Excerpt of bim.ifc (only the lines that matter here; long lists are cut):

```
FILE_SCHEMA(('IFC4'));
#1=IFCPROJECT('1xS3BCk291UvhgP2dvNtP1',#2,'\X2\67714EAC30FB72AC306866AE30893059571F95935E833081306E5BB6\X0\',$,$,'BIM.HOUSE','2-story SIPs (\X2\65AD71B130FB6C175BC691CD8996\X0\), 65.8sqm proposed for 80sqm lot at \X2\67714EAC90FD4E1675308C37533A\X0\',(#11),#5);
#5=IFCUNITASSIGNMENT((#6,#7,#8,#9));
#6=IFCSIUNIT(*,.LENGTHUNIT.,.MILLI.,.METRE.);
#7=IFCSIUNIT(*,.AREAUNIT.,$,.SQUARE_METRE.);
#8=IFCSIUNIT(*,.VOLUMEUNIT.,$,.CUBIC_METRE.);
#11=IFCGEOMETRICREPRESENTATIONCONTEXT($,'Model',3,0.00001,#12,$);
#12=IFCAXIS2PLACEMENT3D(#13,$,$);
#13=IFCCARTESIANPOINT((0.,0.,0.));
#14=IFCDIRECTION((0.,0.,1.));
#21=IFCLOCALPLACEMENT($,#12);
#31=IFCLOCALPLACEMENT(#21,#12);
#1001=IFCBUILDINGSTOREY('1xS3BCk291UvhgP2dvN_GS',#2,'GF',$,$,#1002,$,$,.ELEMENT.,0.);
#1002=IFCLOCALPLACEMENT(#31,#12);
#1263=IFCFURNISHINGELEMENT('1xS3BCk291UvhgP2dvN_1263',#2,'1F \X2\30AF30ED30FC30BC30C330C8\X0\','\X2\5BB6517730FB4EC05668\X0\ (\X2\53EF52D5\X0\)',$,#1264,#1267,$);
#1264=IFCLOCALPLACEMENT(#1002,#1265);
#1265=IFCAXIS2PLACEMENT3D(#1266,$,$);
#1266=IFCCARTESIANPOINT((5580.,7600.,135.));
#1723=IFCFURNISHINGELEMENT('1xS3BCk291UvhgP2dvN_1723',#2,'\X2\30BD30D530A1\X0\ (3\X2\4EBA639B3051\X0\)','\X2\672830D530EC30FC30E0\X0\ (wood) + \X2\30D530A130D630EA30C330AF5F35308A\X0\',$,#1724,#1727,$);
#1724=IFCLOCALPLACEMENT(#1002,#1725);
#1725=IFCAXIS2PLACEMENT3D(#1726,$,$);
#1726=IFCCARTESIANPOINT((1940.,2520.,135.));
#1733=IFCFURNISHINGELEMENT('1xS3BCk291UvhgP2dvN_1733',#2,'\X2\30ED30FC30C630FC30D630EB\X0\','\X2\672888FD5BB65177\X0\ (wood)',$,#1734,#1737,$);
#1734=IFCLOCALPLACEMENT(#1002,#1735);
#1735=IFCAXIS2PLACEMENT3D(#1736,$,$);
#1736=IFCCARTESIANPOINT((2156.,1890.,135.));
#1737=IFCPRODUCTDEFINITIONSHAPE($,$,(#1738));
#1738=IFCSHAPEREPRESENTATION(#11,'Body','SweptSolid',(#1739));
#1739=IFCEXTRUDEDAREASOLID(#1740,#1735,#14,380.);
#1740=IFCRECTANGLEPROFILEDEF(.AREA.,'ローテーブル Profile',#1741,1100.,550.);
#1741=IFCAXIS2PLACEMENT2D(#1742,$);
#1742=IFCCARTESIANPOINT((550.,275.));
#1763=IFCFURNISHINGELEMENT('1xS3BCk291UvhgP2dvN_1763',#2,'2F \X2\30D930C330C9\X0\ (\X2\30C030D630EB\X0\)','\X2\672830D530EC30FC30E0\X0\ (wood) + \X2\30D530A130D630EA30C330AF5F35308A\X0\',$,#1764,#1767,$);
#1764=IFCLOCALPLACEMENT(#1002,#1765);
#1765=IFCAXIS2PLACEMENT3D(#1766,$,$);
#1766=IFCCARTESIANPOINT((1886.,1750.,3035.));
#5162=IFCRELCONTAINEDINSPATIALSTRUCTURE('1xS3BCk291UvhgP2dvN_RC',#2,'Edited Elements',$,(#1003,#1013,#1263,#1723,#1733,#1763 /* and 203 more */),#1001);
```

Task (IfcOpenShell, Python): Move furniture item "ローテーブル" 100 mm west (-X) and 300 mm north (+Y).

```python
import ifcopenshell
import ifcopenshell.api.geometry
import ifcopenshell.util.placement

model = ifcopenshell.open("bim.ifc")

item = model.by_id(1733)
matrix = ifcopenshell.util.placement.get_local_placement(item.ObjectPlacement)
matrix[0, 3] -= 100.0
matrix[1, 3] += 300.0
ifcopenshell.api.geometry.edit_object_placement(model, product=item, matrix=matrix, is_si=False)

print(ifcopenshell.util.placement.get_local_placement(item.ObjectPlacement).round(3) + 0.0)

model.write("bim_edited.ifc")
```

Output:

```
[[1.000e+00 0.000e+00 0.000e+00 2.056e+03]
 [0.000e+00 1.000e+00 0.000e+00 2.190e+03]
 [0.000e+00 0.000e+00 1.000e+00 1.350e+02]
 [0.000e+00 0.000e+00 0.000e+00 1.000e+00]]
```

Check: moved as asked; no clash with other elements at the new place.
